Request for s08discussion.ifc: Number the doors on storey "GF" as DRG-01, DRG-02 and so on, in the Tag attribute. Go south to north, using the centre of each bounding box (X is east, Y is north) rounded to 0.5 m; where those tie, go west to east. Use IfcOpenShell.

First a look at what the model holds.

```python
import ifcopenshell
import ifcopenshell.util.element
import ifcopenshell.util.placement

model = ifcopenshell.open("s08discussion.ifc")
print(model.schema)
storey = next(s for s in model.by_type("IfcBuildingStorey") if s.Name == "GF")
doors = [e for e in ifcopenshell.util.element.get_decomposition(storey) if e.is_a("IfcDoor")]
for e in sorted(doors, key=lambda e: e.id()):
    origin = ifcopenshell.util.placement.get_local_placement(e.ObjectPlacement)[:3, 3]
    print(e.id(), e.Tag, e.Name, origin.round(2) + 0.0, sep=" | ")
```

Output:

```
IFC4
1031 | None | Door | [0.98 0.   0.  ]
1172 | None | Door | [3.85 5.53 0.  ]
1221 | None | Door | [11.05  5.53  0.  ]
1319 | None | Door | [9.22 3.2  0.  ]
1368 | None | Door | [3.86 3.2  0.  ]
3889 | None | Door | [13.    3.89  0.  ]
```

```python
import ifcopenshell
import ifcopenshell.geom
import ifcopenshell.util.element
import ifcopenshell.util.shape

model = ifcopenshell.open("s08discussion.ifc")
settings = ifcopenshell.geom.settings()
settings.set("use-world-coords", True)


def centre(element):
    shape = ifcopenshell.geom.create_shape(settings, element)
    return ifcopenshell.util.shape.get_bbox_centroid(shape.geometry)


storey = next(s for s in model.by_type("IfcBuildingStorey") if s.Name == "GF")
doors = [e for e in ifcopenshell.util.element.get_decomposition(storey) if e.is_a("IfcDoor")]

# Insertion points can sit at a corner or the storey origin, so sort by the geometry (in metres).
centres = {e: centre(e) for e in doors}
doors.sort(key=lambda e: (round(centres[e][1] / 0.5), centres[e][0]))

for i, e in enumerate(doors, start=1):
    number = f"DRG-{i:02d}"
    e.Tag = number
    print(e.id(), number)

model.write("s08discussion_rev.ifc")
```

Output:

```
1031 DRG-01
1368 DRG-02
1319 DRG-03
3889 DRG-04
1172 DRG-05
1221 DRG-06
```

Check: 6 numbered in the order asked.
